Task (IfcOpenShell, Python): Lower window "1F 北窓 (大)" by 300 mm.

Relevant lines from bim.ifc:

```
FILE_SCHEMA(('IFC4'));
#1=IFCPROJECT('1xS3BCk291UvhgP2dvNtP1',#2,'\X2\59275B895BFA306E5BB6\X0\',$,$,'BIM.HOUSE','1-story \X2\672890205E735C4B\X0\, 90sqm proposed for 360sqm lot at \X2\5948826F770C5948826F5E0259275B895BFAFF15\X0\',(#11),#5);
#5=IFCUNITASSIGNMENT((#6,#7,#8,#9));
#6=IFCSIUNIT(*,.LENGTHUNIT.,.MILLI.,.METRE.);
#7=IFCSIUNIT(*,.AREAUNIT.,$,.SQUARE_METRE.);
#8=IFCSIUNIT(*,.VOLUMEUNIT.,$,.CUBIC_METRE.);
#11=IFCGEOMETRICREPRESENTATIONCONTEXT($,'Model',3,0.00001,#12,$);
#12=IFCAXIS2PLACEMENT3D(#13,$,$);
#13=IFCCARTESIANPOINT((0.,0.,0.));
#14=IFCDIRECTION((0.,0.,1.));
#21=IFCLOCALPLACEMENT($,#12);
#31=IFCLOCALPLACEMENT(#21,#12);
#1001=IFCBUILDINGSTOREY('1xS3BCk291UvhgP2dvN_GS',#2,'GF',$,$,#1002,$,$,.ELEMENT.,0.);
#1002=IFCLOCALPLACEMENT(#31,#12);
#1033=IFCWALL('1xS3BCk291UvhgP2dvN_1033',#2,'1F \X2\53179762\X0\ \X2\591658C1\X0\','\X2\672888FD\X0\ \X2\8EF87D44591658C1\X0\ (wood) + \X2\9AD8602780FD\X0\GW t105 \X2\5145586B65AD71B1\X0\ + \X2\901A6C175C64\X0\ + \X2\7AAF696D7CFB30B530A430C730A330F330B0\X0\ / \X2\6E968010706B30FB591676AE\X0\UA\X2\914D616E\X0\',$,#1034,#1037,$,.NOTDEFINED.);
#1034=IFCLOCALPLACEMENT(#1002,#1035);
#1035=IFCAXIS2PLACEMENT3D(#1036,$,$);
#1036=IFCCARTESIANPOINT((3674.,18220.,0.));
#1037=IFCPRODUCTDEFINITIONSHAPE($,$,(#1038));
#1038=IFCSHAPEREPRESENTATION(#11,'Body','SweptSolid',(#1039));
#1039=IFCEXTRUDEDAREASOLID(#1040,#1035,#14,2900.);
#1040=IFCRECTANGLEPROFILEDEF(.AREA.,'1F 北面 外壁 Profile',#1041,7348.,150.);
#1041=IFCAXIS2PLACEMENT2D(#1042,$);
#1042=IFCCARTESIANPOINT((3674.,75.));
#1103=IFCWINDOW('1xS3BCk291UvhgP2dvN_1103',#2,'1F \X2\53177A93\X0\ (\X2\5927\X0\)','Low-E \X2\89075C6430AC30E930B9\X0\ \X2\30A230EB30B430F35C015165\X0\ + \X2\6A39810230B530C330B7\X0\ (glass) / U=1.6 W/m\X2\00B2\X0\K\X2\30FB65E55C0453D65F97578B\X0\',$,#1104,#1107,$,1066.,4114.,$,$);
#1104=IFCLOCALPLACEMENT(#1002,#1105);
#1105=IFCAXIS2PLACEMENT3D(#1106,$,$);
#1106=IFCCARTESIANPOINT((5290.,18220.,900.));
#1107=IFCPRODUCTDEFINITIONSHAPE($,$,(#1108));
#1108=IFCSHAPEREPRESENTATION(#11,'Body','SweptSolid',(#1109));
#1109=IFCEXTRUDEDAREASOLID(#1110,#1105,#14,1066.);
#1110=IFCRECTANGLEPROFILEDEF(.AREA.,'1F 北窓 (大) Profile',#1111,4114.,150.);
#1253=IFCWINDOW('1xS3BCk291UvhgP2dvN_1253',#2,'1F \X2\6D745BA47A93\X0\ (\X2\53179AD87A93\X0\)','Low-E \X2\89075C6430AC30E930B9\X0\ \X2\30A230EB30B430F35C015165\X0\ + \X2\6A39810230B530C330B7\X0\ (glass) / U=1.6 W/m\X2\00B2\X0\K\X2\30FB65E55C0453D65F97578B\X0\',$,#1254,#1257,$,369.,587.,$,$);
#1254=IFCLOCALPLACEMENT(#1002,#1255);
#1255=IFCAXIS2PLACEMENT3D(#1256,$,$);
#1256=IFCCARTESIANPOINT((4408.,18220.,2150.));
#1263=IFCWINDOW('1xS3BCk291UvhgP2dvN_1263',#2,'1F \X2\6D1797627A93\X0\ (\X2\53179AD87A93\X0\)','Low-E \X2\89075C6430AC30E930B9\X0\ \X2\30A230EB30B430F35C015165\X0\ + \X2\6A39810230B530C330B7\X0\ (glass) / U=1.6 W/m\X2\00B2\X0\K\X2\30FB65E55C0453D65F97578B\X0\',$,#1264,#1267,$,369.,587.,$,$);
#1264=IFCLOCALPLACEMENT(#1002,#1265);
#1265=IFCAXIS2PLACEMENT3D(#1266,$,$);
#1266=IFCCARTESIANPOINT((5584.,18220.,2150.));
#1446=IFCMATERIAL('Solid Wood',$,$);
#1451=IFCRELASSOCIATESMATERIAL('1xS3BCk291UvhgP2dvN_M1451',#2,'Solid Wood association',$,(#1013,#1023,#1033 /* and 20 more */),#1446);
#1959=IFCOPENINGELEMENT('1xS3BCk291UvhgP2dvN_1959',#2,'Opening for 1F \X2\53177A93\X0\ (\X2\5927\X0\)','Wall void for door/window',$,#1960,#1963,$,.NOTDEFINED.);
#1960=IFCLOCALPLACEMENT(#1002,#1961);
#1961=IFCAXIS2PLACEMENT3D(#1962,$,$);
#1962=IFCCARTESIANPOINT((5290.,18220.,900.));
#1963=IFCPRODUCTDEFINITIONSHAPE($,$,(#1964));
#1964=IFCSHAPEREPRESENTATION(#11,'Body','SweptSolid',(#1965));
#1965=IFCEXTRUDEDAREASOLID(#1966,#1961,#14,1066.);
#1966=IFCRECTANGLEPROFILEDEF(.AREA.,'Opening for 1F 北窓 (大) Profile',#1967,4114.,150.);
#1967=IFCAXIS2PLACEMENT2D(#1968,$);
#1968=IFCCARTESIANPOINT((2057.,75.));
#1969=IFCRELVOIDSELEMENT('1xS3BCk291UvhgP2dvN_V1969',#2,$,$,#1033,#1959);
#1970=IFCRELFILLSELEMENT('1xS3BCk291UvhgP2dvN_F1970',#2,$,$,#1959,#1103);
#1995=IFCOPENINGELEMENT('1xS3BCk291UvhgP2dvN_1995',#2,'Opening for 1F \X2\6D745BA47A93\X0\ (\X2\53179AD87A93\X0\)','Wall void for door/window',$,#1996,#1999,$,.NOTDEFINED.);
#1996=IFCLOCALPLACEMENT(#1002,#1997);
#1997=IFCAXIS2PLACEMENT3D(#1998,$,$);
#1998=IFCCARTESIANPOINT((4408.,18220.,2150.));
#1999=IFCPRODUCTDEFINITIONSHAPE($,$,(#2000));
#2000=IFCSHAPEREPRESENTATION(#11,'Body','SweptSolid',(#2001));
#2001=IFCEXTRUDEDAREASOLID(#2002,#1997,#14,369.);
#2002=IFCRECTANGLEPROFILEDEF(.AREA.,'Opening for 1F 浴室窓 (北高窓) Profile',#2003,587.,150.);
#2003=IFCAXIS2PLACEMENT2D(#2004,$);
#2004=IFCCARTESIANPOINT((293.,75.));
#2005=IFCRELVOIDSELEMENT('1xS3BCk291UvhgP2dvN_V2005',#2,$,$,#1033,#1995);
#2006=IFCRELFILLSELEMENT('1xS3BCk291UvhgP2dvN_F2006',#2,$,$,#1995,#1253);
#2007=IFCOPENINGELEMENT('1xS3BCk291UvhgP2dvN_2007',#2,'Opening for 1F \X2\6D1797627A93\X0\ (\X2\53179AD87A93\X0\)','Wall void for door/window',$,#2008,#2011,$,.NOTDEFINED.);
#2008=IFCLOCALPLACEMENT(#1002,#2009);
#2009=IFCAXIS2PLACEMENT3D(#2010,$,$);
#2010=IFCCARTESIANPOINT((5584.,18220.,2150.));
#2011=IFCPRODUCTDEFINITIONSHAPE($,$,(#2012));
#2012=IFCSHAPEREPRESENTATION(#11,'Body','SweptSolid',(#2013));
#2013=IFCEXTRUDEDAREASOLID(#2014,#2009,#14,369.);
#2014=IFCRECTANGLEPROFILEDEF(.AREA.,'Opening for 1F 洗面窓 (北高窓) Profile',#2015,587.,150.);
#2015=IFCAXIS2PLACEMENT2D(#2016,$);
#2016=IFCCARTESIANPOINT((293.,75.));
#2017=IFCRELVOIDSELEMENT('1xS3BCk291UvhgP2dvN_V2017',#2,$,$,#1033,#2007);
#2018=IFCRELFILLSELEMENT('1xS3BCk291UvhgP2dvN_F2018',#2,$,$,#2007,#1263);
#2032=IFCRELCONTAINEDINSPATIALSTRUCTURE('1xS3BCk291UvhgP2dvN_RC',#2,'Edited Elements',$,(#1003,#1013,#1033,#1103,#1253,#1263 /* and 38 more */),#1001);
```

```python
import numpy as np
import ifcopenshell
import ifcopenshell.api.geometry
import ifcopenshell.util.placement
import ifcopenshell.util.unit

model = ifcopenshell.open("bim.ifc")
unit_scale = ifcopenshell.util.unit.calculate_unit_scale(model)

window = model.by_id(1103)
opening = window.FillsVoids[0].RelatingOpeningElement
dz = -0.3 / unit_scale

shift = np.array([0.0, 0.0, dz])
# The window is not placed relative to its opening, so move both.
for product in (opening, window):
    matrix = ifcopenshell.util.placement.get_local_placement(product.ObjectPlacement)
    matrix[:3, 3] += shift
    ifcopenshell.api.geometry.edit_object_placement(model, product=product, matrix=matrix, is_si=False)

print(f"moved by {dz * unit_scale:+.3f} m")

model.write("bim_edited.ifc")
```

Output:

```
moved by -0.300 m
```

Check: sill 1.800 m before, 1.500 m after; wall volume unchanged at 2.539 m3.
